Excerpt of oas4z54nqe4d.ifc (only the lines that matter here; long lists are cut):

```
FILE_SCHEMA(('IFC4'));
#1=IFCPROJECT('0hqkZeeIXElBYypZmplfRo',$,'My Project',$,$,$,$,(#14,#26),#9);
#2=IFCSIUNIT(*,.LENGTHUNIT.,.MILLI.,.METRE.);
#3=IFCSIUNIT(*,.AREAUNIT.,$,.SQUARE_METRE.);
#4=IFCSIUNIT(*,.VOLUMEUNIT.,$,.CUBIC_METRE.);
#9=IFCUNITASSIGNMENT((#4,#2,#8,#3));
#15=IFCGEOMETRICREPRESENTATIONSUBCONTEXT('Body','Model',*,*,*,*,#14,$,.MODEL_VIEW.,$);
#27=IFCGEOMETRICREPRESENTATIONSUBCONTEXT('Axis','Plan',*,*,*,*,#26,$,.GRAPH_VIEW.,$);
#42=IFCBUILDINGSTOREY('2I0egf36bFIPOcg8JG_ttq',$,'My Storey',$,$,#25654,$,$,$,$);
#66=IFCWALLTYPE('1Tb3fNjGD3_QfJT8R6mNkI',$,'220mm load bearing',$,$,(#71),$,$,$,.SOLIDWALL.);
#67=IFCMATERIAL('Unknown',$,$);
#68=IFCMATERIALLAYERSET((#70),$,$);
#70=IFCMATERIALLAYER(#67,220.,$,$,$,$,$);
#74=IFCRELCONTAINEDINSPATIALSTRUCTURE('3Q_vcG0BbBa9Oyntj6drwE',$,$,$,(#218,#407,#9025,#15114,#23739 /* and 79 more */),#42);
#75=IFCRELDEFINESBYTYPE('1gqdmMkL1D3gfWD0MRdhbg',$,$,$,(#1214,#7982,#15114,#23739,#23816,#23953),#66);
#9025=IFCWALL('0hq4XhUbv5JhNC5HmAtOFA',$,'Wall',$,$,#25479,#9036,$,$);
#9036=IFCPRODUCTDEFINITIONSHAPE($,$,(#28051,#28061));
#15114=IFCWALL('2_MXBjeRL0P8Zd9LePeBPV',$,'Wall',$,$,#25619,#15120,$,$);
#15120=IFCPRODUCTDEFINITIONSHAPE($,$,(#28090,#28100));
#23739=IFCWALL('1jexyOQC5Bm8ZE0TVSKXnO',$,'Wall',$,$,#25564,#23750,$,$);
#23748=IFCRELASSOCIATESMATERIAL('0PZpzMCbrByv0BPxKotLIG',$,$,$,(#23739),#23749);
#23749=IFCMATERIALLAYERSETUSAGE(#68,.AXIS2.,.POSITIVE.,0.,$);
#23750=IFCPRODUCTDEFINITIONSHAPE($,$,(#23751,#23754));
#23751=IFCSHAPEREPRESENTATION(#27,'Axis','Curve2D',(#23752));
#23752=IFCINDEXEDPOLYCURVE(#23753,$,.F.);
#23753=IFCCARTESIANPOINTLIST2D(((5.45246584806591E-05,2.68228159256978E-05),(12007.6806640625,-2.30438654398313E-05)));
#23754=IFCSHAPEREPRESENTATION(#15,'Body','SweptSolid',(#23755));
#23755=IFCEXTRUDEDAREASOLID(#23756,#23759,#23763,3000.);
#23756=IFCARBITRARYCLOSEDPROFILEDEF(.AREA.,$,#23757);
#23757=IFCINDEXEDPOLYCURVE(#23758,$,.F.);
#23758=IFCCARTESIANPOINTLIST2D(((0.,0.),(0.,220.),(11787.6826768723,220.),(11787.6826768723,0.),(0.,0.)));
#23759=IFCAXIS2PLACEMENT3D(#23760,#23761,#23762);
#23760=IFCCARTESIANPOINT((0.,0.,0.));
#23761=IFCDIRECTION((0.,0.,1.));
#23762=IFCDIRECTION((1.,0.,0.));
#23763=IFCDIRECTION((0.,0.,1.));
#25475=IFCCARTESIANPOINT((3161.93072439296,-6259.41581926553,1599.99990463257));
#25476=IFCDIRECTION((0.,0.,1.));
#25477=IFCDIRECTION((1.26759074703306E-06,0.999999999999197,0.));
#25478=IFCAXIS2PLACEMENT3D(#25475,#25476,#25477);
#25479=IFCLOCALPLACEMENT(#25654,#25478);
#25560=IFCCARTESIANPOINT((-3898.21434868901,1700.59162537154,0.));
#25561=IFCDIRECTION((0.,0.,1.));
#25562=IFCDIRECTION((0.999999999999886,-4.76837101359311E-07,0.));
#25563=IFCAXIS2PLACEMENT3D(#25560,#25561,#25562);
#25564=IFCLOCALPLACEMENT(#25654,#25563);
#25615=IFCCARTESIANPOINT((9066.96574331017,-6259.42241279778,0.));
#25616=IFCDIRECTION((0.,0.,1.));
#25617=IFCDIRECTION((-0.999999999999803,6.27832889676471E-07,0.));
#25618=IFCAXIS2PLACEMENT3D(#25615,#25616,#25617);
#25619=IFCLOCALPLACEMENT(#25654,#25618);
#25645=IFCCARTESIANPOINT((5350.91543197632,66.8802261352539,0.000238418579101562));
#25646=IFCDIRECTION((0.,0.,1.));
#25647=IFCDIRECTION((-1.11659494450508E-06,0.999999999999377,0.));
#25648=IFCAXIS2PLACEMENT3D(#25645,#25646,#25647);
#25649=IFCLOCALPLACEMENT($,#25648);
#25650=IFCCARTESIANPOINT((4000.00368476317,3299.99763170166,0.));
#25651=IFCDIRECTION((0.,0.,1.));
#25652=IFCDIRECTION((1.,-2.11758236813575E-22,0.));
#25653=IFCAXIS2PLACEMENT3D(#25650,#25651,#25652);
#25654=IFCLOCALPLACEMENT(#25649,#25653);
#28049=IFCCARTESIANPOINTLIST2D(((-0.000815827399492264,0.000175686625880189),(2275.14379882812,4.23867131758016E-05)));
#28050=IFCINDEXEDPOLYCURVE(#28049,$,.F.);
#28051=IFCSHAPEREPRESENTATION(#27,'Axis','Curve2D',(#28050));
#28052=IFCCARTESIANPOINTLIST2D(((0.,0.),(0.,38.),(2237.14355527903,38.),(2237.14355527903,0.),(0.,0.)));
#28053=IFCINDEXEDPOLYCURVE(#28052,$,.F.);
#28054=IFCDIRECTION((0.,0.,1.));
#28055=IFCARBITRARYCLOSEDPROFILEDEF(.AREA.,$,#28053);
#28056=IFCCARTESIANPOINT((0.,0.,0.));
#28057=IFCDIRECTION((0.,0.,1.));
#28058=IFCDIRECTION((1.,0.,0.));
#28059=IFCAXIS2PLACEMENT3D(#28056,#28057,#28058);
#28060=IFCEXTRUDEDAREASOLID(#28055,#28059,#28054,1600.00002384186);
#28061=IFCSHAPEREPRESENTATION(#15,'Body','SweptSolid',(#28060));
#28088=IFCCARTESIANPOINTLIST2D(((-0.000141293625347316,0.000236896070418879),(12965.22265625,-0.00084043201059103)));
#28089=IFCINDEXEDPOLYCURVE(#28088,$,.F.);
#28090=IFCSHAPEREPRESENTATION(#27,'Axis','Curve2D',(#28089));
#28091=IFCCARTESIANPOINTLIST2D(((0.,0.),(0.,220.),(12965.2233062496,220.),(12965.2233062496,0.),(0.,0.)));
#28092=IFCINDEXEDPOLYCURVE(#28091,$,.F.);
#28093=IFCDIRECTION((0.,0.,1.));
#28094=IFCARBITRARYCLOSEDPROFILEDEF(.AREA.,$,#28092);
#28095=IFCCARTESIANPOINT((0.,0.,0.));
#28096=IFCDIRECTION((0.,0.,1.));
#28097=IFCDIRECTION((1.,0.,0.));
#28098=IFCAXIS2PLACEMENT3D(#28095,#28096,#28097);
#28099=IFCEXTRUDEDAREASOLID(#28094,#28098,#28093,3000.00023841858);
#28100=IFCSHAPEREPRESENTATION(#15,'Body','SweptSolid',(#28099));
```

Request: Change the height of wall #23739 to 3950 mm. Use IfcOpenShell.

```python
import ifcopenshell
import ifcopenshell.geom
import ifcopenshell.util.representation
import ifcopenshell.util.shape

model = ifcopenshell.open("oas4z54nqe4d.ifc")
settings = ifcopenshell.geom.settings()


def volume(element):
    """Net volume in cubic metres, openings subtracted."""
    shape = ifcopenshell.geom.create_shape(settings, element)
    return ifcopenshell.util.shape.get_volume(shape.geometry)


wall = model.by_id(23739)
before = volume(wall)

body = ifcopenshell.util.representation.get_representation(wall, "Model", "Body")
solid = body.Items[0]
old_height = solid.Depth
solid.Depth = 3950.0
after = volume(wall)

print(f"height {old_height:g} -> {solid.Depth:g}, volume {before:.3f} -> {after:.3f} m3")

model.write("oas4z54nqe4d-out.ifc")
```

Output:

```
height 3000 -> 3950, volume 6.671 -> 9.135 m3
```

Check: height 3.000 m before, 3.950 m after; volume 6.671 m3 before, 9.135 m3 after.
